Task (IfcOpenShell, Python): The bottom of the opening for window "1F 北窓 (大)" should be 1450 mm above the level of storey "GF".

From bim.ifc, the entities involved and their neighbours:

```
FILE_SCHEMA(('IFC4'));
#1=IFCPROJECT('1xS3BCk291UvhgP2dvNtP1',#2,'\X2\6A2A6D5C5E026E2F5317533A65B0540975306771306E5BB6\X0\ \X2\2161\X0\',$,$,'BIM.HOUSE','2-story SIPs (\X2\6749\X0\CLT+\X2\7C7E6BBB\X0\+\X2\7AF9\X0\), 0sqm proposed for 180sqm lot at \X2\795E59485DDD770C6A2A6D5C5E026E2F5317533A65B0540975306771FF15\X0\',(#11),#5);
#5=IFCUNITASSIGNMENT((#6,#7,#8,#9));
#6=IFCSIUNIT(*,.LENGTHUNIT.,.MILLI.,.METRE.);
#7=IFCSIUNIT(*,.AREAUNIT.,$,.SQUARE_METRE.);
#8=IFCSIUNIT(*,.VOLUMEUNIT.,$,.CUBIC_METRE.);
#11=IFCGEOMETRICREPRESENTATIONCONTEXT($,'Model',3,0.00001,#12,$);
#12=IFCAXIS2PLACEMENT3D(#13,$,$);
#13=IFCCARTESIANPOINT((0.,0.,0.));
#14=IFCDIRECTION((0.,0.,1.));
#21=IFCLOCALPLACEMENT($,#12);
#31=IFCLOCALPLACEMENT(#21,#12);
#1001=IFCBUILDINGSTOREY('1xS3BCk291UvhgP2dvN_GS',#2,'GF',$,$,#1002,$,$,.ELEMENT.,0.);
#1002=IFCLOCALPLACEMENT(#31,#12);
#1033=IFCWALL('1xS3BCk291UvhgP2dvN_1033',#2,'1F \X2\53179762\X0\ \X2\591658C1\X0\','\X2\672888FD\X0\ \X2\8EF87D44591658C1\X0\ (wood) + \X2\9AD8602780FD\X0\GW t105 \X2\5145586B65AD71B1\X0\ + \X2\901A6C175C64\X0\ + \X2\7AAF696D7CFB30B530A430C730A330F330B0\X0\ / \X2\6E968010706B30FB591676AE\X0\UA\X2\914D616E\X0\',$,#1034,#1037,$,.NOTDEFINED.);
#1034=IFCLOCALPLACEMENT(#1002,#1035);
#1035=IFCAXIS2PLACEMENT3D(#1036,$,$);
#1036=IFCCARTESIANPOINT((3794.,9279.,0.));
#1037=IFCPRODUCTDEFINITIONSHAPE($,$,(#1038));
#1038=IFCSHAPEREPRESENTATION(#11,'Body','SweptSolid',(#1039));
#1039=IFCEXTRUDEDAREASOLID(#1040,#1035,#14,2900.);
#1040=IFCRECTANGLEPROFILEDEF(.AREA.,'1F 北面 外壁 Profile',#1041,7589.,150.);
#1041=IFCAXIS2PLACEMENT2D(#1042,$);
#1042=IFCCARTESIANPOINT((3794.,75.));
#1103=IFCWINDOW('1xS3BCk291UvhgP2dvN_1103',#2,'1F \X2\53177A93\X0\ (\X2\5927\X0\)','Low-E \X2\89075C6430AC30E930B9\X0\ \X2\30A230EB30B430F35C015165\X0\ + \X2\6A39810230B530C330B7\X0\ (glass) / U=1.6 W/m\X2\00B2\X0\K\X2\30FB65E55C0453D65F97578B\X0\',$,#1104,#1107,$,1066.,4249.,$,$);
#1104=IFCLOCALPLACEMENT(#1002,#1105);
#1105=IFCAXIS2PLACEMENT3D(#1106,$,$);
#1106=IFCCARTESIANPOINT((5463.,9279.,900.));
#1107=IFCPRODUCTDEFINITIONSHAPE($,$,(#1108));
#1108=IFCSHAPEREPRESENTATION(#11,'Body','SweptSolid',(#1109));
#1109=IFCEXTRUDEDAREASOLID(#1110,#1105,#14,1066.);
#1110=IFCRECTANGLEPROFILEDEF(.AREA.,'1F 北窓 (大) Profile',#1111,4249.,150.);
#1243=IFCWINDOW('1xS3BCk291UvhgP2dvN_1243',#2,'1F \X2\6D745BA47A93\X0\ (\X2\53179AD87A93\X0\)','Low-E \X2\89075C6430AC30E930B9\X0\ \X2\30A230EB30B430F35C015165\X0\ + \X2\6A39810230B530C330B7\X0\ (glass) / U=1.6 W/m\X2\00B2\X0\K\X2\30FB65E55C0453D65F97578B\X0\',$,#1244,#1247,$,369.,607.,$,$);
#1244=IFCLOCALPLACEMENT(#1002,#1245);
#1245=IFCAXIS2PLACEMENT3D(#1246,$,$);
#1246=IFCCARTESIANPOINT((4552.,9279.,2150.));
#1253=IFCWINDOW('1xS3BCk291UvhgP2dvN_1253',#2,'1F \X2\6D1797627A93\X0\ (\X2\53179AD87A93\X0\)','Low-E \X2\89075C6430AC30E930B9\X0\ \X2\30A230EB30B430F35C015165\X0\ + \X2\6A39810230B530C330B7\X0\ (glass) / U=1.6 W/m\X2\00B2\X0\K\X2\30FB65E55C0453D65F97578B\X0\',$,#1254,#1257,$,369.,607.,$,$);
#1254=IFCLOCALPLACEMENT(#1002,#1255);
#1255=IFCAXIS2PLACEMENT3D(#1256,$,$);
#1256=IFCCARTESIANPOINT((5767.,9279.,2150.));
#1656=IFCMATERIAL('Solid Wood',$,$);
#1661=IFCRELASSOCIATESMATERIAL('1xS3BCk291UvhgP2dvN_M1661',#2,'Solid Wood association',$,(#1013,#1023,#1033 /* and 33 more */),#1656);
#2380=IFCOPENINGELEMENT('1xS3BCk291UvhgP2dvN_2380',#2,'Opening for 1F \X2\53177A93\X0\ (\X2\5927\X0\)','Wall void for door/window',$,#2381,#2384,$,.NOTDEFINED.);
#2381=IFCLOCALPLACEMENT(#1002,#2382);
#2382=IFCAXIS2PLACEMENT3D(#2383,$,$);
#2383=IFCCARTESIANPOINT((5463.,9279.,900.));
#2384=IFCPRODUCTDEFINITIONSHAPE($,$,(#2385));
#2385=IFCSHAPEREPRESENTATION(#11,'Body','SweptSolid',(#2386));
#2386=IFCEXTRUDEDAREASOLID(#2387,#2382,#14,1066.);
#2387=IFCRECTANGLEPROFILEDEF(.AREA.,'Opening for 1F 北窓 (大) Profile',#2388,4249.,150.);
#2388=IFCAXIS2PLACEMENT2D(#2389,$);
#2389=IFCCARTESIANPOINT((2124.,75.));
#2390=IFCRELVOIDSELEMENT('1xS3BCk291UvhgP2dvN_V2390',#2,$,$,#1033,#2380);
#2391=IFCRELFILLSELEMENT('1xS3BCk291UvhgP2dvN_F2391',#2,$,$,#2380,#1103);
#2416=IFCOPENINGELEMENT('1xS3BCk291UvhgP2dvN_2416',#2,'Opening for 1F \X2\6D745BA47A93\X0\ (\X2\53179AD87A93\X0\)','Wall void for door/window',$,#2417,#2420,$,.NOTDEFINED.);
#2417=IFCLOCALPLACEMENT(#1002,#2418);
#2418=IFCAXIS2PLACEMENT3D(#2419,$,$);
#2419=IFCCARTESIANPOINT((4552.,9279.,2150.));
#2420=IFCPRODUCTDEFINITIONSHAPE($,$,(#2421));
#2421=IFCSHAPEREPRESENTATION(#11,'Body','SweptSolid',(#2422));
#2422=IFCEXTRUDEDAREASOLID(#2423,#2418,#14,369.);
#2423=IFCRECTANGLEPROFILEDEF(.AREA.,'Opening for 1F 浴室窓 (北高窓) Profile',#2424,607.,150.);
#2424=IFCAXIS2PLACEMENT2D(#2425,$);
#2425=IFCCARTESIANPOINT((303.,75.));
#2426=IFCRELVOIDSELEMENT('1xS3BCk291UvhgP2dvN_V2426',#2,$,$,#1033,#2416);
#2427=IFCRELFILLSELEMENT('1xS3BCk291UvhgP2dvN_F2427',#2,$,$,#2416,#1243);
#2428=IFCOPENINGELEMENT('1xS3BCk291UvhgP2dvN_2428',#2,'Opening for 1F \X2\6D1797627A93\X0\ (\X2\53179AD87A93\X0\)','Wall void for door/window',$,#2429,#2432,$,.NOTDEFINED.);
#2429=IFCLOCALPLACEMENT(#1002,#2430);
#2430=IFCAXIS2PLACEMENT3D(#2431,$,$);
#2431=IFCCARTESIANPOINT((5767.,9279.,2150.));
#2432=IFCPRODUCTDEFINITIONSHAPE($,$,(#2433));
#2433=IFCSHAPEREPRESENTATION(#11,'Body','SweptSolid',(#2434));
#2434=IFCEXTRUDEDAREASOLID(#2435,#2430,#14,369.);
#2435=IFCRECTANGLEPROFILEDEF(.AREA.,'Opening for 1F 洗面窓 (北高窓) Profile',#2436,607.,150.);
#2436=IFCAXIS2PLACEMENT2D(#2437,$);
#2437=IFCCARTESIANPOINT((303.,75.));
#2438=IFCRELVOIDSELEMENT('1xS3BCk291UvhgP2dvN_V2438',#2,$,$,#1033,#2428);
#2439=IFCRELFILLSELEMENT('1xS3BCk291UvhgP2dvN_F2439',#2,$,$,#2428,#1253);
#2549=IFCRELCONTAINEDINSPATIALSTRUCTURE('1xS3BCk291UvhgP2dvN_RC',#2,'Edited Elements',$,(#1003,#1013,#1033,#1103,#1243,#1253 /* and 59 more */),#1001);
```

```python
import numpy as np
import ifcopenshell
import ifcopenshell.api.geometry
import ifcopenshell.geom
import ifcopenshell.util.element
import ifcopenshell.util.placement
import ifcopenshell.util.shape
import ifcopenshell.util.unit

model = ifcopenshell.open("bim.ifc")
unit_scale = ifcopenshell.util.unit.calculate_unit_scale(model)

window = model.by_guid("1xS3BCk291UvhgP2dvN_1103")
opening = window.FillsVoids[0].RelatingOpeningElement
storey = ifcopenshell.util.element.get_container(window, ifc_class="IfcBuildingStorey")
level = ifcopenshell.util.placement.get_local_placement(storey.ObjectPlacement)[2, 3]

# The opening's origin need not be at the sill, so measure its lowest point.
shape = ifcopenshell.geom.create_shape(ifcopenshell.geom.settings(), opening)
bottom = ifcopenshell.util.shape.get_shape_bottom_elevation(shape, shape.geometry) / unit_scale
dz = level + 1450.0 - bottom

shift = np.array([0.0, 0.0, dz])
# The window is not placed relative to its opening, so move both.
for product in (opening, window):
    matrix = ifcopenshell.util.placement.get_local_placement(product.ObjectPlacement)
    matrix[:3, 3] += shift
    ifcopenshell.api.geometry.edit_object_placement(model, product=product, matrix=matrix, is_si=False)

print(f"moved by {dz * unit_scale:+.3f} m")

model.write("bim-out.ifc")
```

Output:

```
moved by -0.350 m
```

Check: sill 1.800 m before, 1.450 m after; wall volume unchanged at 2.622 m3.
